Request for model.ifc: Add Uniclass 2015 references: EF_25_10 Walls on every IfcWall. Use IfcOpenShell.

First a look at what the model holds.

```python
import ifcopenshell

model = ifcopenshell.open("model.ifc")
print(model.schema)
print("classifications:", [c.Name for c in model.by_type("IfcClassification")])
for ifc_class in ("IfcDoor", "IfcRoof", "IfcStair", "IfcWall", "IfcWindow"):
    print(ifc_class, len(model.by_type(ifc_class)))
```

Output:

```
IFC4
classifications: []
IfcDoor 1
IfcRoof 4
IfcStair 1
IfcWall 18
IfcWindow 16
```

```python
import ifcopenshell
import ifcopenshell.api.classification

model = ifcopenshell.open("model.ifc")

system = ifcopenshell.api.classification.add_classification(model, classification="Uniclass 2015")

codes = {
    "IfcWall": ("EF_25_10", "Walls"),
}
for ifc_class, (code, name) in codes.items():
    products = model.by_type(ifc_class)
    ifcopenshell.api.classification.add_reference(
        model, products=products, classification=system, identification=code, name=name
    )
    print(code, len(products))

model.write("model-out.ifc")
```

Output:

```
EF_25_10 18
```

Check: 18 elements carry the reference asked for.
